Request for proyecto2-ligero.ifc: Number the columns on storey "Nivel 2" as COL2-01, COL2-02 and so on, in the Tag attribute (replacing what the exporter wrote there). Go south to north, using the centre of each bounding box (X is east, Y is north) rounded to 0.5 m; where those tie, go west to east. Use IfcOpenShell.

First a look at what the model holds.

```python
import ifcopenshell
import ifcopenshell.util.element
import ifcopenshell.util.placement

model = ifcopenshell.open("proyecto2-ligero.ifc")
print(model.schema)
storey = next(s for s in model.by_type("IfcBuildingStorey") if s.Name == "Nivel 2")
columns = [e for e in ifcopenshell.util.element.get_decomposition(storey) if e.is_a("IfcColumn")]
for e in sorted(columns, key=lambda e: e.id()):
    origin = ifcopenshell.util.placement.get_local_placement(e.ObjectPlacement)[:3, 3]
    print(e.id(), e.Tag, e.Name, origin.round(2) + 0.0, sep=" | ")
```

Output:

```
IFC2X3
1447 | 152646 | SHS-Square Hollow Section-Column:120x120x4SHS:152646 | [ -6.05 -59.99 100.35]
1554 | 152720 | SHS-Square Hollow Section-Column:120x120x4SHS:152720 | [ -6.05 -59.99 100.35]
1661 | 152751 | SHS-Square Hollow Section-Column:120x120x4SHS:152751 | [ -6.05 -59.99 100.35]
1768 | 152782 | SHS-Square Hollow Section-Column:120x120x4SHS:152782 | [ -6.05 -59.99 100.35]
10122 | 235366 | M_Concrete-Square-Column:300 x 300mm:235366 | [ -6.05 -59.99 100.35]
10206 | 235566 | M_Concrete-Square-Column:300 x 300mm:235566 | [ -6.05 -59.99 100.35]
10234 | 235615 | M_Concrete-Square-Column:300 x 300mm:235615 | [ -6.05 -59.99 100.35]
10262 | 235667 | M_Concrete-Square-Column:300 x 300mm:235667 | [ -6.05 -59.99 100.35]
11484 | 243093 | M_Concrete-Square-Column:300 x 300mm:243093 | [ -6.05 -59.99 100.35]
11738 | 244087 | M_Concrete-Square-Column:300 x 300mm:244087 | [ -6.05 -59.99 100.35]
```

```python
import ifcopenshell
import ifcopenshell.geom
import ifcopenshell.util.element
import ifcopenshell.util.shape

model = ifcopenshell.open("proyecto2-ligero.ifc")
settings = ifcopenshell.geom.settings()
settings.set("use-world-coords", True)


def centre(element):
    shape = ifcopenshell.geom.create_shape(settings, element)
    return ifcopenshell.util.shape.get_bbox_centroid(shape.geometry)


storey = next(s for s in model.by_type("IfcBuildingStorey") if s.Name == "Nivel 2")
columns = [e for e in ifcopenshell.util.element.get_decomposition(storey) if e.is_a("IfcColumn")]

# Insertion points can sit at a corner or the storey origin, so sort by the geometry (in metres).
centres = {e: centre(e) for e in columns}
columns.sort(key=lambda e: (round(centres[e][1] / 0.5), centres[e][0]))

for i, e in enumerate(columns, start=1):
    number = f"COL2-{i:02d}"
    e.Tag = number
    print(e.id(), number)

model.write("proyecto2-ligero_rev.ifc")
```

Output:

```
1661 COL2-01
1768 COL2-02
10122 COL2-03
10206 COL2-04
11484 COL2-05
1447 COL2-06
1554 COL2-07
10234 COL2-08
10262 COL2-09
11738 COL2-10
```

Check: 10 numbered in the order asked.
